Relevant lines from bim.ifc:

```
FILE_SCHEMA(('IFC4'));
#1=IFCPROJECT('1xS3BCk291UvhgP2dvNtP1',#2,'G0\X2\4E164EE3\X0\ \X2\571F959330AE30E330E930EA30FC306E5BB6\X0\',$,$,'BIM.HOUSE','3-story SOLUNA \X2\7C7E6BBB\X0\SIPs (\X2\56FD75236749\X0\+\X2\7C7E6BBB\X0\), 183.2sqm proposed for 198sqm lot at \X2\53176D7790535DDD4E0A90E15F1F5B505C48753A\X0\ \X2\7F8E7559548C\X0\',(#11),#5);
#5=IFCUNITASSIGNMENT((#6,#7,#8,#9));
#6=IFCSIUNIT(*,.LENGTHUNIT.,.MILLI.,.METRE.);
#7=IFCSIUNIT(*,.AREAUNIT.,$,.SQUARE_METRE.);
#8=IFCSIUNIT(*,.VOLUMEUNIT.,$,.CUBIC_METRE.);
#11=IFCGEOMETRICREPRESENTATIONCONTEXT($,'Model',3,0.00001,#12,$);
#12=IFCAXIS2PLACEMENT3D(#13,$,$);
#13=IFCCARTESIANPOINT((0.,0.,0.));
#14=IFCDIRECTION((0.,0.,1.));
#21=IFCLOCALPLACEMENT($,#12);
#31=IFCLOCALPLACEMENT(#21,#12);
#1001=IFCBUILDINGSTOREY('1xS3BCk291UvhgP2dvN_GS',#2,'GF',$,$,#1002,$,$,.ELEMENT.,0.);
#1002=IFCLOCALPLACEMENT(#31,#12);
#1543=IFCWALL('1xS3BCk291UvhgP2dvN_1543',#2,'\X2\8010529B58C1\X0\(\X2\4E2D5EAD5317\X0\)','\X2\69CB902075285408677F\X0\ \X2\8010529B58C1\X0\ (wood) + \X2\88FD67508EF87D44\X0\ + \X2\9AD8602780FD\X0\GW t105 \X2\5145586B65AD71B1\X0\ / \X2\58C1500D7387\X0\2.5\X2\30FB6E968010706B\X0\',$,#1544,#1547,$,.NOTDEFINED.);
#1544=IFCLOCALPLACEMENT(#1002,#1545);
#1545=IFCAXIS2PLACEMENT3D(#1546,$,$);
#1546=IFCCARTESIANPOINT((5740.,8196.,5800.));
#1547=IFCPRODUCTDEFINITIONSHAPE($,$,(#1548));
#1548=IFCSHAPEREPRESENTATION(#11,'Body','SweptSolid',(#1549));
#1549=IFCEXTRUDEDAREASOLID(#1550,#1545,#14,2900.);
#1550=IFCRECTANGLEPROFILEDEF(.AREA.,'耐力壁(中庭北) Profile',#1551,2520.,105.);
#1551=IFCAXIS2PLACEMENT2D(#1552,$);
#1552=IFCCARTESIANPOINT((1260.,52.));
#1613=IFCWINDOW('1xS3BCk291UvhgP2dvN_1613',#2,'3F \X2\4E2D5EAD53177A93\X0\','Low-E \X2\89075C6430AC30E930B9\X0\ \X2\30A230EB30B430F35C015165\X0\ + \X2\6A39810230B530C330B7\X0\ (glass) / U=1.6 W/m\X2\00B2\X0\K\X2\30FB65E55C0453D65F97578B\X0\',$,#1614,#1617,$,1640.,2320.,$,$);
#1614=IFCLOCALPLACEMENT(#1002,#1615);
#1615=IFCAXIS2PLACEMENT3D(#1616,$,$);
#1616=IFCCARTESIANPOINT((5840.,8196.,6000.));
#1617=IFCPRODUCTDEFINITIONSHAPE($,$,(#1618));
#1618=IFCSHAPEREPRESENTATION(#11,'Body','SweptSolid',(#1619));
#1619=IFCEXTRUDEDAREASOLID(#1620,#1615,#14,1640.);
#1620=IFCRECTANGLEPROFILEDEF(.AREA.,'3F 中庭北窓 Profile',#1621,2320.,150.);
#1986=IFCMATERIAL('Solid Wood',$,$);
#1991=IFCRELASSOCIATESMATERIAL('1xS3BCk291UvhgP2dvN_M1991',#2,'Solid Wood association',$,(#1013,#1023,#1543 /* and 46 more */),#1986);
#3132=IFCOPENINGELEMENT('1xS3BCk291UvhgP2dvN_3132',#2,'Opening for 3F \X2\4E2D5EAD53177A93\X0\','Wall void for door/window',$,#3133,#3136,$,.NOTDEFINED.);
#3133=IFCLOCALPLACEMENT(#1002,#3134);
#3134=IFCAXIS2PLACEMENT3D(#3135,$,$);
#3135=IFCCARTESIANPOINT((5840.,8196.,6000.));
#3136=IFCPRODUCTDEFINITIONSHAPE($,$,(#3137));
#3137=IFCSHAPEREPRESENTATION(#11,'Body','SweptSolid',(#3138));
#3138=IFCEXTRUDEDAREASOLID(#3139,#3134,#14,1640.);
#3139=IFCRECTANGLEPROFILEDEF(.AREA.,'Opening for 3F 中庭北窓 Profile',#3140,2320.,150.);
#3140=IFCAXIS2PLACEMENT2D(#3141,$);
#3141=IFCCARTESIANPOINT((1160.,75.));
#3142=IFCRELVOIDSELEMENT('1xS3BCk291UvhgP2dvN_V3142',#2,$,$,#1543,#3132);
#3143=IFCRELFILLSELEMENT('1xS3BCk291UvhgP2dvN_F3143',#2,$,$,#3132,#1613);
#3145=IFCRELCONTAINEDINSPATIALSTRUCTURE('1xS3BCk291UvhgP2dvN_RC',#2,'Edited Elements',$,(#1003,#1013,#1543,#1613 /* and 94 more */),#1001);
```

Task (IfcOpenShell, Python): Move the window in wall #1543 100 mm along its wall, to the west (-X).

```python
import ifcopenshell
import ifcopenshell.api.geometry
import ifcopenshell.util.placement
import ifcopenshell.util.unit

model = ifcopenshell.open("bim.ifc")
unit_scale = ifcopenshell.util.unit.calculate_unit_scale(model)

window = model.by_id(1613)
opening = window.FillsVoids[0].RelatingOpeningElement
wall = opening.VoidsElements[0].RelatingBuildingElement

wall_matrix = ifcopenshell.util.placement.get_local_placement(wall.ObjectPlacement)
shift = wall_matrix[:3, 0] * -0.1 / unit_scale
before = ifcopenshell.util.placement.get_local_placement(window.ObjectPlacement)[:3, 3].copy()

# The window is not placed relative to its opening, so move both.
for product in (opening, window):
    matrix = ifcopenshell.util.placement.get_local_placement(product.ObjectPlacement)
    matrix[:3, 3] += shift
    ifcopenshell.api.geometry.edit_object_placement(model, product=product, matrix=matrix, is_si=False)

after = ifcopenshell.util.placement.get_local_placement(window.ObjectPlacement)[:3, 3]
print("window moved by", (after - before).round(3) + 0.0)

model.write("bim-out.ifc")
```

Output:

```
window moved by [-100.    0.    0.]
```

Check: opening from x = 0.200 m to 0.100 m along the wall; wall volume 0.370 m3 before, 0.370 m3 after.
